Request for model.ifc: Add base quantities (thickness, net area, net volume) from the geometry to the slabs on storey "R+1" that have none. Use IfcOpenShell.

First a look at what the model holds.

```python
import ifcopenshell
import ifcopenshell.util.element
import ifcopenshell.util.unit

model = ifcopenshell.open("model.ifc")
print(model.schema)
for unit_type in ("LENGTHUNIT", "AREAUNIT", "VOLUMEUNIT"):
    print(unit_type, ifcopenshell.util.unit.calculate_unit_scale(model, unit_type))
storey = next(s for s in model.by_type("IfcBuildingStorey") if s.Name == "R+1")
slabs = [e for e in ifcopenshell.util.element.get_decomposition(storey) if e.is_a("IfcSlab")]
for e in sorted(slabs, key=lambda e: e.id()):
    print(e.id(), e.is_a(), e.Name, list(ifcopenshell.util.element.get_psets(e, qtos_only=True)), sep=" | ")
```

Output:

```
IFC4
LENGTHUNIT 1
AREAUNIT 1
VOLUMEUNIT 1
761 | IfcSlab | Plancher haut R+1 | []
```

```python
import ifcopenshell
import ifcopenshell.api.pset
import ifcopenshell.geom
import ifcopenshell.util.element
import ifcopenshell.util.shape
import ifcopenshell.util.unit

model = ifcopenshell.open("model.ifc")
unit_scale = ifcopenshell.util.unit.calculate_unit_scale(model)
area_scale = ifcopenshell.util.unit.calculate_unit_scale(model, "AREAUNIT")
volume_scale = ifcopenshell.util.unit.calculate_unit_scale(model, "VOLUMEUNIT")
settings = ifcopenshell.geom.settings()

storey = next(s for s in model.by_type("IfcBuildingStorey") if s.Name == "R+1")
slabs = [e for e in ifcopenshell.util.element.get_decomposition(storey) if e.is_a("IfcSlab")]

for e in sorted(slabs, key=lambda e: e.id()):
    if ifcopenshell.util.element.get_psets(e, qtos_only=True, should_inherit=False):
        continue
    # Geometry comes back in metres, in the element's own axes.
    shape = ifcopenshell.geom.create_shape(settings, e)
    values = {
        "Width": ifcopenshell.util.shape.get_z(shape.geometry) / unit_scale,
        "NetArea": ifcopenshell.util.shape.get_footprint_area(shape.geometry) / area_scale,
        "NetVolume": ifcopenshell.util.shape.get_volume(shape.geometry) / volume_scale,
    }
    qto = ifcopenshell.api.pset.add_qto(model, product=e, name="Qto_SlabBaseQuantities")
    ifcopenshell.api.pset.edit_qto(model, qto=qto, properties=values)
    print(e.id(), {k: round(v, 3) for k, v in values.items()})

model.write("model-out.ifc")
```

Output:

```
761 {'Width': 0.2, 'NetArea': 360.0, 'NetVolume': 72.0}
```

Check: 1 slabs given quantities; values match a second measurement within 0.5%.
